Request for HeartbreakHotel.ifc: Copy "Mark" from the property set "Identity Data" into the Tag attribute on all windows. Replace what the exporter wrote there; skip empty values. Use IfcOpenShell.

First a look at what the model holds.

```python
import ifcopenshell
import ifcopenshell.util.element

model = ifcopenshell.open("HeartbreakHotel.ifc")
print(model.schema)
windows = model.by_type("IfcWindow")
print(len(windows), "windows")
for e in windows[:8]:
    source = ifcopenshell.util.element.get_pset(e, "Identity Data", "Mark")
    target = e.Tag
    print(e.id(), repr(source), repr(target), sep=" | ")
```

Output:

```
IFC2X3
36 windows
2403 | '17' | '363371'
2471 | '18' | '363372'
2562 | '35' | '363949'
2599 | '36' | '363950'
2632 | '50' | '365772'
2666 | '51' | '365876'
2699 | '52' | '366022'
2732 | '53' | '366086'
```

```python
import ifcopenshell
import ifcopenshell.util.element

model = ifcopenshell.open("HeartbreakHotel.ifc")

count = 0
for e in model.by_type("IfcWindow"):
    value = ifcopenshell.util.element.get_pset(e, "Identity Data", "Mark")
    current = e.Tag
    if not value or not value.strip() or current == value:
        continue
    e.Tag = value
    count += 1

print(count, "windows updated")

model.write("HeartbreakHotel_edited.ifc")
```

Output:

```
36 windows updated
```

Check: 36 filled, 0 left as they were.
